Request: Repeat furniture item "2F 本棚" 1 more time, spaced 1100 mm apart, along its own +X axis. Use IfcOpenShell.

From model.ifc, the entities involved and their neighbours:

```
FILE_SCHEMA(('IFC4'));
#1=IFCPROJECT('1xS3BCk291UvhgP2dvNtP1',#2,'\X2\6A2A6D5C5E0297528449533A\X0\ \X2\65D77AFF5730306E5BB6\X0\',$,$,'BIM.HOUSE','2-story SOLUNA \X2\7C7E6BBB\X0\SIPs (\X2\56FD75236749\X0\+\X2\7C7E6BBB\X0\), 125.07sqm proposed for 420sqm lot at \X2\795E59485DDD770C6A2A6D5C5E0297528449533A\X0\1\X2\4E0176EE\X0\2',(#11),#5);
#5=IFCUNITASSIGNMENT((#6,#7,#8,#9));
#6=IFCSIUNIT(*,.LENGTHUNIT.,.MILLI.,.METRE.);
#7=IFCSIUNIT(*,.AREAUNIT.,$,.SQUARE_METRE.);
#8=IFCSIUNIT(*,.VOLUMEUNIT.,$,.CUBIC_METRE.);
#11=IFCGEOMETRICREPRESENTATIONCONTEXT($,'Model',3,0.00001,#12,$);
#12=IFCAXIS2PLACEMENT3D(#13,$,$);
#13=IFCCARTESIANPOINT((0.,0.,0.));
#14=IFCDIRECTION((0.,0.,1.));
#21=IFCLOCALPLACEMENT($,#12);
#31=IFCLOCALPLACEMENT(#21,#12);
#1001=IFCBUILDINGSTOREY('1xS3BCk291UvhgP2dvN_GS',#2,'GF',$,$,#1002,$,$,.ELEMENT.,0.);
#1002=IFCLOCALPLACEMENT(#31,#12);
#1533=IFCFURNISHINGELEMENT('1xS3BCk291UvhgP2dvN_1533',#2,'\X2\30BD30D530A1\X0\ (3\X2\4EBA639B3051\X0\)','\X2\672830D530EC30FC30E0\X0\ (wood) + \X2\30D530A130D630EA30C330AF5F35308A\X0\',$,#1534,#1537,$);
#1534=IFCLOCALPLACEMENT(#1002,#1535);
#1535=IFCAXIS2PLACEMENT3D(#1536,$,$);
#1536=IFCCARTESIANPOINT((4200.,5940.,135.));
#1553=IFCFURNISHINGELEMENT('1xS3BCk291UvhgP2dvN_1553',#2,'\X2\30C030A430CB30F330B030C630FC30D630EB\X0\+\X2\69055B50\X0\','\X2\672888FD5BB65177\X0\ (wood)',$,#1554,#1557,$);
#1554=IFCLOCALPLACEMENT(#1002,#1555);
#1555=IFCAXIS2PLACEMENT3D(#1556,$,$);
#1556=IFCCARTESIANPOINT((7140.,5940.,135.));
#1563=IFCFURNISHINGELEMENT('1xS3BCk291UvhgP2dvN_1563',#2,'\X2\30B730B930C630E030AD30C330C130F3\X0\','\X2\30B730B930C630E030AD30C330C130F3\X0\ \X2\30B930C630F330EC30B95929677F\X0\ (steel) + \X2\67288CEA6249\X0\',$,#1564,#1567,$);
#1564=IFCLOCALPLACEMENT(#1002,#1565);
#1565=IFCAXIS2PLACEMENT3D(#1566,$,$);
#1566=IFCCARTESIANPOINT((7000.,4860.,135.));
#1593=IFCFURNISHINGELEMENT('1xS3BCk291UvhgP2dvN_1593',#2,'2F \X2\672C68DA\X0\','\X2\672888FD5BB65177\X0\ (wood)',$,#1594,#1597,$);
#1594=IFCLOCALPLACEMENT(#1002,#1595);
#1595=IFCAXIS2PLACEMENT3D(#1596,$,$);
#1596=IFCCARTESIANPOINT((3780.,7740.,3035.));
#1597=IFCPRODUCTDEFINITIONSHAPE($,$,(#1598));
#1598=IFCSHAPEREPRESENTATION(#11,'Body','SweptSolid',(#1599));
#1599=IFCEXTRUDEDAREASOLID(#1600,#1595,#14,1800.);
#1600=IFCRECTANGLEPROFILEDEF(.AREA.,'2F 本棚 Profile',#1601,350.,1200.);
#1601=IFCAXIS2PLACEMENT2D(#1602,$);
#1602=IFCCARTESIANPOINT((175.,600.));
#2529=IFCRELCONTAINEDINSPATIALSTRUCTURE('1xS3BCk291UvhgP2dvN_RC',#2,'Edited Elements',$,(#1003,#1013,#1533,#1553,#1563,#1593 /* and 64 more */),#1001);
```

```python
import ifcopenshell
import ifcopenshell.api.geometry
import ifcopenshell.api.root
import ifcopenshell.util.element
import ifcopenshell.util.placement
import ifcopenshell.util.unit

model = ifcopenshell.open("model.ifc")
unit_scale = ifcopenshell.util.unit.calculate_unit_scale(model)


def reuse_history(source, copy):
    """copy_class also copies each property set's owner history, people and application; keep the originals."""
    for rel in copy.IsDefinedBy:
        if rel.is_a("IfcRelDefinesByProperties") and (history := rel.RelatingPropertyDefinition.OwnerHistory):
            rel.RelatingPropertyDefinition.OwnerHistory = source.OwnerHistory
            ifcopenshell.util.element.remove_deep2(model, history)


source = model.by_guid("1xS3BCk291UvhgP2dvN_1593")
base = ifcopenshell.util.placement.get_local_placement(source.ObjectPlacement)
step = base[:3, 0] * 1.1 / unit_scale

for i in range(1, 2):
    copy = ifcopenshell.api.root.copy_class(model, product=source)
    copy.Representation = ifcopenshell.util.element.copy_deep(
        model, source.Representation, exclude=["IfcGeometricRepresentationContext", "IfcRepresentationMap"]
    )
    reuse_history(source, copy)
    matrix = base.copy()
    matrix[:3, 3] += i * step
    print("added at", matrix[:3, 3].round(3) + 0.0)
    ifcopenshell.api.geometry.edit_object_placement(model, product=copy, matrix=matrix, is_si=False)

model.write("model_v2.ifc")
```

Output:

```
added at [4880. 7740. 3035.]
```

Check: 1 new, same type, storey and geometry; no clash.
